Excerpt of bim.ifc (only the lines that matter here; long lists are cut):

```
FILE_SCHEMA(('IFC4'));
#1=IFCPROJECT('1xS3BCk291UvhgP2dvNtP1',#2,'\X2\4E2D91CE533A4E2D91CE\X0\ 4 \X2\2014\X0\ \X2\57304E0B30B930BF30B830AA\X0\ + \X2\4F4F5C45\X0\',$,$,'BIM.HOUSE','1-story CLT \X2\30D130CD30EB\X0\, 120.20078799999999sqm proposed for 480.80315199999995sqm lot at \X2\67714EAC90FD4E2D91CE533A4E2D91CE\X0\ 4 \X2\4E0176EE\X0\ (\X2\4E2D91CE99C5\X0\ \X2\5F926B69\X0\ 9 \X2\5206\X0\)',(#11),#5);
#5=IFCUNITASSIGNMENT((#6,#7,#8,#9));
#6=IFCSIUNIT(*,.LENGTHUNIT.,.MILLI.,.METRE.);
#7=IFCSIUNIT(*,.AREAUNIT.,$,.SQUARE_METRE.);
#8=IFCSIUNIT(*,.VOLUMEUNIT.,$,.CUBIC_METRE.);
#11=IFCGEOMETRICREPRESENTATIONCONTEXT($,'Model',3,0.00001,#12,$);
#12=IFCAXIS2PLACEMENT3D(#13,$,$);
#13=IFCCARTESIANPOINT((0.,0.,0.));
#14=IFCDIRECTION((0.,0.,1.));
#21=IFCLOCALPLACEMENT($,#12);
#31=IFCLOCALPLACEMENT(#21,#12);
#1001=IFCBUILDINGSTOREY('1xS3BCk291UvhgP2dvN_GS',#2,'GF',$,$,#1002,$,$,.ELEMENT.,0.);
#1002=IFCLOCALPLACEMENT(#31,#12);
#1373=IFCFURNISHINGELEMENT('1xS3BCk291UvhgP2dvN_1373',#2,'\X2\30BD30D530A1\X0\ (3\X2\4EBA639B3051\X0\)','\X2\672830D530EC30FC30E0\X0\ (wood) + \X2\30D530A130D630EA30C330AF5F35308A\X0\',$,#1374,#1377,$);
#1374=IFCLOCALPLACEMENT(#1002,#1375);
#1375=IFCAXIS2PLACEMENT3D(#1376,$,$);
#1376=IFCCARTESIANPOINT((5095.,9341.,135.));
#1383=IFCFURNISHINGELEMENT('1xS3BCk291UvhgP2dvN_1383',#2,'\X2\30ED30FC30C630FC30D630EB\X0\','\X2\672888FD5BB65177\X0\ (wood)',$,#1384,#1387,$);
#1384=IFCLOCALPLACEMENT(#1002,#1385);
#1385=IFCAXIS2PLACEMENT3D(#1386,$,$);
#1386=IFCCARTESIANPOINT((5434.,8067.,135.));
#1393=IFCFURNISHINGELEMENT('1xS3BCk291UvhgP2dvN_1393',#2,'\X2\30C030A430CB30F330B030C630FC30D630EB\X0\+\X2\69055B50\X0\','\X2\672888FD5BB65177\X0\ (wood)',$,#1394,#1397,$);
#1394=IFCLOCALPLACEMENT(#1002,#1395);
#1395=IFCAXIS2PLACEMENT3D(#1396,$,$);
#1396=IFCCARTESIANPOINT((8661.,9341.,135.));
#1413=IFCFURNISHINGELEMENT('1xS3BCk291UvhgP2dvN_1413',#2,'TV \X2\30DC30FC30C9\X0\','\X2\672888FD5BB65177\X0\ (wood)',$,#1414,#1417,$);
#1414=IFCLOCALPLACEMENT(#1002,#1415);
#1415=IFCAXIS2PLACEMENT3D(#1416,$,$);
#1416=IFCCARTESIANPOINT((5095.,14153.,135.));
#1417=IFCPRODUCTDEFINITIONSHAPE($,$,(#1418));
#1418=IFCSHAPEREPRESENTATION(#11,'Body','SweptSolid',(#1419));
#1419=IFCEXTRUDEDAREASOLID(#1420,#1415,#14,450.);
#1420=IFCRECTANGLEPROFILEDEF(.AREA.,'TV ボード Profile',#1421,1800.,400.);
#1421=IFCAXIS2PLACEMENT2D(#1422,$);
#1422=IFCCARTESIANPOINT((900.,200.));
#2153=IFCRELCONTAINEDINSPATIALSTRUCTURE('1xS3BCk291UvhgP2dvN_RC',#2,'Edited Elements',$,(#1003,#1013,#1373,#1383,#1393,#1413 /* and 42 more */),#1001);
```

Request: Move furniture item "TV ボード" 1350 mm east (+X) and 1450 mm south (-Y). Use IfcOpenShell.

```python
import ifcopenshell
import ifcopenshell.api.geometry
import ifcopenshell.util.placement
import ifcopenshell.util.unit

model = ifcopenshell.open("bim.ifc")
unit_scale = ifcopenshell.util.unit.calculate_unit_scale(model)

item = model.by_guid("1xS3BCk291UvhgP2dvN_1413")
matrix = ifcopenshell.util.placement.get_local_placement(item.ObjectPlacement)
matrix[0, 3] += 1.35 / unit_scale
matrix[1, 3] -= 1.45 / unit_scale
ifcopenshell.api.geometry.edit_object_placement(model, product=item, matrix=matrix, is_si=False)

print(ifcopenshell.util.placement.get_local_placement(item.ObjectPlacement).round(3) + 0.0)

model.write("bim_v2.ifc")
```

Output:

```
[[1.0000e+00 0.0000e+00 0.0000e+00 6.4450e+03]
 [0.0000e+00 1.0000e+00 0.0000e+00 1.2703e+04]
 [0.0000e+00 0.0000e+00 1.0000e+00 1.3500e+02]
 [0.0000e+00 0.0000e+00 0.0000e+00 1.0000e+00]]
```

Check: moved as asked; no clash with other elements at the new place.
